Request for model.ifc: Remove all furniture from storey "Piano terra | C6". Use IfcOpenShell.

First a look at what the model holds.

```python
import ifcopenshell
import ifcopenshell.util.element

model = ifcopenshell.open("model.ifc")
print(model.schema)
storey = next(s for s in model.by_type("IfcBuildingStorey") if s.Name == "Piano terra | C6")
furniture = [e for e in ifcopenshell.util.element.get_decomposition(storey) if e.is_a("IfcFurnishingElement")]
seen = {}
for e in furniture:
    element_type = ifcopenshell.util.element.get_type(e)
    name = element_type.Name if element_type not in (None, e) else None
    seen[name] = seen.get(name, 0) + 1
for name, count in sorted(seen.items(), key=str):
    print(count, "x", name)
```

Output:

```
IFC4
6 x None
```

```python
import ifcopenshell
import ifcopenshell.api.root
import ifcopenshell.util.element

model = ifcopenshell.open("model.ifc")

storey = next(s for s in model.by_type("IfcBuildingStorey") if s.Name == "Piano terra | C6")
furniture = [e for e in ifcopenshell.util.element.get_decomposition(storey) if e.is_a("IfcFurnishingElement")]

for e in furniture:
    ifcopenshell.api.root.remove_product(model, product=e)
print(len(furniture), "removed")

model.write("model_updated.ifc")
```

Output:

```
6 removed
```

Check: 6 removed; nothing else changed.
